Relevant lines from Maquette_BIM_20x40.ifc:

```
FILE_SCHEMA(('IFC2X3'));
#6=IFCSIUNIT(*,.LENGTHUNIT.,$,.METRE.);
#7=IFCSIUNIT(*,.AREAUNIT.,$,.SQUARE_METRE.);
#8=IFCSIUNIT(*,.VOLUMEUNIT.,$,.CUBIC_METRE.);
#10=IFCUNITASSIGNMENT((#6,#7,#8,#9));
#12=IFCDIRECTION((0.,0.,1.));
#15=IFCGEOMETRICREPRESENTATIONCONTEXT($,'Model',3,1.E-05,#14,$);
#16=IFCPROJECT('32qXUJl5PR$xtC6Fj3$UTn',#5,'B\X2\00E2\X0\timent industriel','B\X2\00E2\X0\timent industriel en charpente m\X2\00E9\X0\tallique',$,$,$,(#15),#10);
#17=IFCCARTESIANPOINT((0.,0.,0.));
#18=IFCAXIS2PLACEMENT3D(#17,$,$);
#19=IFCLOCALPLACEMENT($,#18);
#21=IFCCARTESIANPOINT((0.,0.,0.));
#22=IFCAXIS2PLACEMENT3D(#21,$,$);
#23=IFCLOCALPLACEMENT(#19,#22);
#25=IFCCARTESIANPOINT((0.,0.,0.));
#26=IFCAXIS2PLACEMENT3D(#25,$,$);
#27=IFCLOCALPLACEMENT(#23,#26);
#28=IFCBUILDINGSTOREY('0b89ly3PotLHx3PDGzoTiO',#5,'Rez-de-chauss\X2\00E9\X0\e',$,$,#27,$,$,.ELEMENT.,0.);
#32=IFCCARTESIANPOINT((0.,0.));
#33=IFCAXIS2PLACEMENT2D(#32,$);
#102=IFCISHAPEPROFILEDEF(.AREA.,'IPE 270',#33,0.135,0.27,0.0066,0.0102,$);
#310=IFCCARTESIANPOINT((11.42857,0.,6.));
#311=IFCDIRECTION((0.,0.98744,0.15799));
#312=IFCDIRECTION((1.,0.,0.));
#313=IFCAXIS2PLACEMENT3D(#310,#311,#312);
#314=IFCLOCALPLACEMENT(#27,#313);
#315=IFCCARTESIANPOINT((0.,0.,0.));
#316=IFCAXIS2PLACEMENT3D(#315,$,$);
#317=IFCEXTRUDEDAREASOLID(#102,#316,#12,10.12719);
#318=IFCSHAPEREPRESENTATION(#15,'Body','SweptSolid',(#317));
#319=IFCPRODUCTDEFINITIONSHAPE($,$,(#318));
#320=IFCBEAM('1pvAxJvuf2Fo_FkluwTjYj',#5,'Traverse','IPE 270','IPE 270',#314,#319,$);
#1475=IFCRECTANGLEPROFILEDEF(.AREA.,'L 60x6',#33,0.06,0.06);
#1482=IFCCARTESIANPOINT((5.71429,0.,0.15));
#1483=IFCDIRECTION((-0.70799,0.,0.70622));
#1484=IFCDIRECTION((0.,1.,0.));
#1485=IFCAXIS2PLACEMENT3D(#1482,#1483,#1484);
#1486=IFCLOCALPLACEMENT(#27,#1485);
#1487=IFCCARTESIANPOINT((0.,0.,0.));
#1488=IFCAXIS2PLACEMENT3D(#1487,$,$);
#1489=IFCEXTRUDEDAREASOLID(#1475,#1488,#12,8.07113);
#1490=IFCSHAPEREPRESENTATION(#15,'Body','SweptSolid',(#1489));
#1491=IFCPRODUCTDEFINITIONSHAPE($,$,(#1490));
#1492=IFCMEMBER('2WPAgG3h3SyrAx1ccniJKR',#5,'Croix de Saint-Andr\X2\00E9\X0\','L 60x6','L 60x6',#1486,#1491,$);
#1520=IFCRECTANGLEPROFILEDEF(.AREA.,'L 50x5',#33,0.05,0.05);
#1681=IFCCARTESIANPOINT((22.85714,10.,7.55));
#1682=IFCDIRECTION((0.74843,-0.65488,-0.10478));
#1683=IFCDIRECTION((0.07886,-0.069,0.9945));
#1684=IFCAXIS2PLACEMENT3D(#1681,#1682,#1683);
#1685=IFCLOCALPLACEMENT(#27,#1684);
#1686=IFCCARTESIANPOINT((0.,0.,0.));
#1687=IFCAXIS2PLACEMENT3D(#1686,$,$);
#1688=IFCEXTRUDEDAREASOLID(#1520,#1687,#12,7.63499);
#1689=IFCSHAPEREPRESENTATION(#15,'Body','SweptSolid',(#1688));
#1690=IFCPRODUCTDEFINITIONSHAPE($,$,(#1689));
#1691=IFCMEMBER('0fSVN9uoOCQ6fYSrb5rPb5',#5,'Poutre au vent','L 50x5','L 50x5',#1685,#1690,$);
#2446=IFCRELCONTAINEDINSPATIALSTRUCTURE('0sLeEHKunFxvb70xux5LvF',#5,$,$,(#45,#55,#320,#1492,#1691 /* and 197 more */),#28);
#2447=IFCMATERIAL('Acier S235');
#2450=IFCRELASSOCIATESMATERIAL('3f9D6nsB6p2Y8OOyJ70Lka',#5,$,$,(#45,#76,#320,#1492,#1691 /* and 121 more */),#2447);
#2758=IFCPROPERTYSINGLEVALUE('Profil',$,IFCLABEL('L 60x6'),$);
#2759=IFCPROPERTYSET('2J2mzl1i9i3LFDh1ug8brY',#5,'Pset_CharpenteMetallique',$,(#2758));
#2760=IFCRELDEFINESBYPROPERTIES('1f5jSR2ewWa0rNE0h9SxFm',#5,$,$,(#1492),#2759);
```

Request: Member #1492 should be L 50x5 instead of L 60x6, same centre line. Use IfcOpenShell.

```python
import ifcopenshell
import ifcopenshell.api.pset
import ifcopenshell.util.element

model = ifcopenshell.open("Maquette_BIM_20x40.ifc")

member = model.by_id(1492)
source = next(p for p in model.by_type("IfcRectangleProfileDef") if p.ProfileName == "L 50x5")

body = next(r for r in member.Representation.Representations if r.RepresentationIdentifier == "Body")
solid = body.Items[0]
old_profile = solid.SweptArea

# Copy the section's sizes but keep this member's own profile position.
profile = ifcopenshell.util.element.copy(model, source)
profile.Position = old_profile.Position
solid.SweptArea = profile
if not model.get_total_inverses(old_profile):
    ifcopenshell.util.element.remove_deep2(model, old_profile)
member.Description = member.Description.replace("L 60x6", "L 50x5")
member.ObjectType = member.ObjectType.replace("L 60x6", "L 50x5")
pset = model.by_id(ifcopenshell.util.element.get_pset(member, "Pset_CharpenteMetallique", should_inherit=False)["id"])
ifcopenshell.api.pset.edit_pset(model, pset=pset, properties={"Profil": "L 50x5"})

print(solid.SweptArea)

model.write("Maquette_BIM_20x40_rev.ifc")
```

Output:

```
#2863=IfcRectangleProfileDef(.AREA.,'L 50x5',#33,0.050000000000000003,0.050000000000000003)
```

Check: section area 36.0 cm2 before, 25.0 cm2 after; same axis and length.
